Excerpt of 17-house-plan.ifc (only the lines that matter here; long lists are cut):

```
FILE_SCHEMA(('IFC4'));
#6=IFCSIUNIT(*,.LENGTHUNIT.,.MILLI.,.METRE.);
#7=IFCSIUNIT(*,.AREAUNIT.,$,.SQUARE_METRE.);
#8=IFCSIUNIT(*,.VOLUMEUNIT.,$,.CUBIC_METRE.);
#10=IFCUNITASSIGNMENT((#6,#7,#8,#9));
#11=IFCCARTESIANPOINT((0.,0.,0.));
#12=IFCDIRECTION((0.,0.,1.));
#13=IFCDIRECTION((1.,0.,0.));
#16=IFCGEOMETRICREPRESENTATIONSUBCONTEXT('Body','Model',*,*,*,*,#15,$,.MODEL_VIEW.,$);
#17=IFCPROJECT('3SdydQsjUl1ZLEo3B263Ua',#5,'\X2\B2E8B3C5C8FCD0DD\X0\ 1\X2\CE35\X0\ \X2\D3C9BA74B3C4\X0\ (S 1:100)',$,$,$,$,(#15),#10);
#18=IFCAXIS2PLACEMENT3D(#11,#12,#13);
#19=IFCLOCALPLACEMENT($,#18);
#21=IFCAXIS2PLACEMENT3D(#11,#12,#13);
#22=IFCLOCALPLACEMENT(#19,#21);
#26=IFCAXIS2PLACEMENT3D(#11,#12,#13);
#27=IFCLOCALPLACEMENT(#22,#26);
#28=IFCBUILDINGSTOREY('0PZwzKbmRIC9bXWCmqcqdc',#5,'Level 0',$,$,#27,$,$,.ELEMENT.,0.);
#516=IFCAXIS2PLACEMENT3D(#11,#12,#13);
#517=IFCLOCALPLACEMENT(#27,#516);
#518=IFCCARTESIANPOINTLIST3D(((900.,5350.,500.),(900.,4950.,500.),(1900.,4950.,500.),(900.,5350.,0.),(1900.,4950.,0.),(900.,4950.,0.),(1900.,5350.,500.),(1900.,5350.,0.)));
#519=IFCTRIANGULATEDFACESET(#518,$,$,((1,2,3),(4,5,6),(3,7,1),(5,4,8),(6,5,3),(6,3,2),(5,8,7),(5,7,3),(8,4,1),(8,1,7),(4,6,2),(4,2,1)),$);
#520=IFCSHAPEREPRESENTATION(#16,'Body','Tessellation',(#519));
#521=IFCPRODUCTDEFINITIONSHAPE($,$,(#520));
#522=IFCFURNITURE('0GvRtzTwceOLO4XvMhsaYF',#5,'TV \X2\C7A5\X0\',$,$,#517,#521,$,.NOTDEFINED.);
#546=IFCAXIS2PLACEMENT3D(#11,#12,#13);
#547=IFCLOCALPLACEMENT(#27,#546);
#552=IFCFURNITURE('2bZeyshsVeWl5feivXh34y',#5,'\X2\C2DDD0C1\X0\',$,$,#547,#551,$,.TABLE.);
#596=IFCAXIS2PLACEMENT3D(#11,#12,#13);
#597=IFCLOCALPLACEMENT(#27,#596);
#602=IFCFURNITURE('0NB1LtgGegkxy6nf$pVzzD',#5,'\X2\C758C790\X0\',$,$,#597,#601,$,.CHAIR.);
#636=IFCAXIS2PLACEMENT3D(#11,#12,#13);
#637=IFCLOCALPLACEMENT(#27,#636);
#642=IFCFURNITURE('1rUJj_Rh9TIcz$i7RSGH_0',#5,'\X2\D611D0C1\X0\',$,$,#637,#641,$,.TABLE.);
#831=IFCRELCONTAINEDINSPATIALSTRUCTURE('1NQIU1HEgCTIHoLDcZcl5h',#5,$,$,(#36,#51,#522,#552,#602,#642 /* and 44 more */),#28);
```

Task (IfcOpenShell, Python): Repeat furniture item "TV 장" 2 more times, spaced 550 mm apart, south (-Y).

```python
import numpy as np
import ifcopenshell
import ifcopenshell.api.geometry
import ifcopenshell.api.root
import ifcopenshell.util.element
import ifcopenshell.util.placement
import ifcopenshell.util.unit

model = ifcopenshell.open("17-house-plan.ifc")
unit_scale = ifcopenshell.util.unit.calculate_unit_scale(model)


def reuse_history(source, copy):
    """copy_class also copies each property set's owner history, people and application; keep the originals."""
    for rel in copy.IsDefinedBy:
        if rel.is_a("IfcRelDefinesByProperties") and (history := rel.RelatingPropertyDefinition.OwnerHistory):
            rel.RelatingPropertyDefinition.OwnerHistory = source.OwnerHistory
            ifcopenshell.util.element.remove_deep2(model, history)


source = model.by_guid("0GvRtzTwceOLO4XvMhsaYF")
base = ifcopenshell.util.placement.get_local_placement(source.ObjectPlacement)
step = np.array([0.0, -1.0, 0.0]) * 0.55 / unit_scale

for i in range(1, 3):
    copy = ifcopenshell.api.root.copy_class(model, product=source)
    copy.Representation = ifcopenshell.util.element.copy_deep(
        model, source.Representation, exclude=["IfcGeometricRepresentationContext", "IfcRepresentationMap"]
    )
    reuse_history(source, copy)
    matrix = base.copy()
    matrix[:3, 3] += i * step
    print("added at", matrix[:3, 3].round(3) + 0.0)
    ifcopenshell.api.geometry.edit_object_placement(model, product=copy, matrix=matrix, is_si=False)

model.write("17-house-plan_updated.ifc")
```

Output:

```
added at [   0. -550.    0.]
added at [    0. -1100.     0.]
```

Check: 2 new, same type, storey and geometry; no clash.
